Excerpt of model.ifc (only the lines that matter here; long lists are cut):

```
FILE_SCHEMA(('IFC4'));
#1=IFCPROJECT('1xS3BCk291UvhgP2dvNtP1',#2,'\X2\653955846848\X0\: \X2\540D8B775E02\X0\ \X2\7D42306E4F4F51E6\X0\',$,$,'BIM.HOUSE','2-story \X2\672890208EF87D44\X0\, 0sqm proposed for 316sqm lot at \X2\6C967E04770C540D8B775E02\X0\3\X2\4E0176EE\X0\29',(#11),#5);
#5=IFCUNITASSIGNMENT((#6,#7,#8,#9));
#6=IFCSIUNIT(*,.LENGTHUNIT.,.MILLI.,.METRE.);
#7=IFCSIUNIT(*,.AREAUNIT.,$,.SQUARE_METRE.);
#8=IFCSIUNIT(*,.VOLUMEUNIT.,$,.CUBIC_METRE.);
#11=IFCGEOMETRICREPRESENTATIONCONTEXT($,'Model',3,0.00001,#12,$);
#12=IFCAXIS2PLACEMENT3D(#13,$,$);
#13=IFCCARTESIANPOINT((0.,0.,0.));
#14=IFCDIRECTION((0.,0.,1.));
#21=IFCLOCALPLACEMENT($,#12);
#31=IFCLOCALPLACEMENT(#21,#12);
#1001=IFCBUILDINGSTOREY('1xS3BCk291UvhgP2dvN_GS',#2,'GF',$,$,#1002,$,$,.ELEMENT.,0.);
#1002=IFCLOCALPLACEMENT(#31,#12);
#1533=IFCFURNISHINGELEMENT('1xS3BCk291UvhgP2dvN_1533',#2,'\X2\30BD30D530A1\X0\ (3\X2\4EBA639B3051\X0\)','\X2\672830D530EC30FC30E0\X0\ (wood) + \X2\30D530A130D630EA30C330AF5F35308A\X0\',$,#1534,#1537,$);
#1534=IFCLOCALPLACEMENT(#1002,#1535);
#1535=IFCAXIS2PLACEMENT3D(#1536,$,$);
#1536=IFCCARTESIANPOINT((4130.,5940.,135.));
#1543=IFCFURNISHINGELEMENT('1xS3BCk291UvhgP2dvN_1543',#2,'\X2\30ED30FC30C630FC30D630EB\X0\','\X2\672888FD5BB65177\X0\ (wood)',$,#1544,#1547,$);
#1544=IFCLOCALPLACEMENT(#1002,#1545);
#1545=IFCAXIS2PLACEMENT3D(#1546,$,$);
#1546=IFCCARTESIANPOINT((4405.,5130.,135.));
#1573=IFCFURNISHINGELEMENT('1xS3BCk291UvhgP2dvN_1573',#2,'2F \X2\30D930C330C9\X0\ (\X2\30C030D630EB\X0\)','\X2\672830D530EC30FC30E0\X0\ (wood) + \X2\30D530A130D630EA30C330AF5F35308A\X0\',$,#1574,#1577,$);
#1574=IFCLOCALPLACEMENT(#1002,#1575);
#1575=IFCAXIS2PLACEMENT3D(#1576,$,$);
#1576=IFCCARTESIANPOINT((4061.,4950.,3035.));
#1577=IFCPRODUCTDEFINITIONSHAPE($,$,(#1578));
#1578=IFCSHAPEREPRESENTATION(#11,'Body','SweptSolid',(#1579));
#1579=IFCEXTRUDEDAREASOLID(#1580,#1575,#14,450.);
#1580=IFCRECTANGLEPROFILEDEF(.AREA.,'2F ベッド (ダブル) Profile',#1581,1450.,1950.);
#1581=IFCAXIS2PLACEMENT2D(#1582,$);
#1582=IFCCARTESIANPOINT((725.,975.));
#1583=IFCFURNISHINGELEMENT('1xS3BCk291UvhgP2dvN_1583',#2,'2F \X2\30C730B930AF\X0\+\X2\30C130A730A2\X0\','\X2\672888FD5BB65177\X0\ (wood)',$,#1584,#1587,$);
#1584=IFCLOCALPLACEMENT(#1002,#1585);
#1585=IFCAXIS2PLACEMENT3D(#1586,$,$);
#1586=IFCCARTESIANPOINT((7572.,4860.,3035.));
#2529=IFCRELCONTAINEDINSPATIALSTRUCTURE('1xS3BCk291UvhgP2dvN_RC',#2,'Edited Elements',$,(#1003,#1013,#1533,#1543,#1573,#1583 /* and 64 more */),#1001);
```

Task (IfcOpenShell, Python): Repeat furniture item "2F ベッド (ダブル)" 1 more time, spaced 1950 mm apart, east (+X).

```python
import numpy as np
import ifcopenshell
import ifcopenshell.api.geometry
import ifcopenshell.api.root
import ifcopenshell.util.element
import ifcopenshell.util.placement

model = ifcopenshell.open("model.ifc")


def reuse_history(source, copy):
    """copy_class also copies each property set's owner history, people and application; keep the originals."""
    for rel in copy.IsDefinedBy:
        if rel.is_a("IfcRelDefinesByProperties") and (history := rel.RelatingPropertyDefinition.OwnerHistory):
            rel.RelatingPropertyDefinition.OwnerHistory = source.OwnerHistory
            ifcopenshell.util.element.remove_deep2(model, history)


source = model.by_id(1573)
base = ifcopenshell.util.placement.get_local_placement(source.ObjectPlacement)
step = np.array([1.0, 0.0, 0.0]) * 1950.0

for i in range(1, 2):
    copy = ifcopenshell.api.root.copy_class(model, product=source)
    copy.Representation = ifcopenshell.util.element.copy_deep(
        model, source.Representation, exclude=["IfcGeometricRepresentationContext", "IfcRepresentationMap"]
    )
    reuse_history(source, copy)
    matrix = base.copy()
    matrix[:3, 3] += i * step
    print("added at", matrix[:3, 3].round(3) + 0.0)
    ifcopenshell.api.geometry.edit_object_placement(model, product=copy, matrix=matrix, is_si=False)

model.write("model_rev.ifc")
```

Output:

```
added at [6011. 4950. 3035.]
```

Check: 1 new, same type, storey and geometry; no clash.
